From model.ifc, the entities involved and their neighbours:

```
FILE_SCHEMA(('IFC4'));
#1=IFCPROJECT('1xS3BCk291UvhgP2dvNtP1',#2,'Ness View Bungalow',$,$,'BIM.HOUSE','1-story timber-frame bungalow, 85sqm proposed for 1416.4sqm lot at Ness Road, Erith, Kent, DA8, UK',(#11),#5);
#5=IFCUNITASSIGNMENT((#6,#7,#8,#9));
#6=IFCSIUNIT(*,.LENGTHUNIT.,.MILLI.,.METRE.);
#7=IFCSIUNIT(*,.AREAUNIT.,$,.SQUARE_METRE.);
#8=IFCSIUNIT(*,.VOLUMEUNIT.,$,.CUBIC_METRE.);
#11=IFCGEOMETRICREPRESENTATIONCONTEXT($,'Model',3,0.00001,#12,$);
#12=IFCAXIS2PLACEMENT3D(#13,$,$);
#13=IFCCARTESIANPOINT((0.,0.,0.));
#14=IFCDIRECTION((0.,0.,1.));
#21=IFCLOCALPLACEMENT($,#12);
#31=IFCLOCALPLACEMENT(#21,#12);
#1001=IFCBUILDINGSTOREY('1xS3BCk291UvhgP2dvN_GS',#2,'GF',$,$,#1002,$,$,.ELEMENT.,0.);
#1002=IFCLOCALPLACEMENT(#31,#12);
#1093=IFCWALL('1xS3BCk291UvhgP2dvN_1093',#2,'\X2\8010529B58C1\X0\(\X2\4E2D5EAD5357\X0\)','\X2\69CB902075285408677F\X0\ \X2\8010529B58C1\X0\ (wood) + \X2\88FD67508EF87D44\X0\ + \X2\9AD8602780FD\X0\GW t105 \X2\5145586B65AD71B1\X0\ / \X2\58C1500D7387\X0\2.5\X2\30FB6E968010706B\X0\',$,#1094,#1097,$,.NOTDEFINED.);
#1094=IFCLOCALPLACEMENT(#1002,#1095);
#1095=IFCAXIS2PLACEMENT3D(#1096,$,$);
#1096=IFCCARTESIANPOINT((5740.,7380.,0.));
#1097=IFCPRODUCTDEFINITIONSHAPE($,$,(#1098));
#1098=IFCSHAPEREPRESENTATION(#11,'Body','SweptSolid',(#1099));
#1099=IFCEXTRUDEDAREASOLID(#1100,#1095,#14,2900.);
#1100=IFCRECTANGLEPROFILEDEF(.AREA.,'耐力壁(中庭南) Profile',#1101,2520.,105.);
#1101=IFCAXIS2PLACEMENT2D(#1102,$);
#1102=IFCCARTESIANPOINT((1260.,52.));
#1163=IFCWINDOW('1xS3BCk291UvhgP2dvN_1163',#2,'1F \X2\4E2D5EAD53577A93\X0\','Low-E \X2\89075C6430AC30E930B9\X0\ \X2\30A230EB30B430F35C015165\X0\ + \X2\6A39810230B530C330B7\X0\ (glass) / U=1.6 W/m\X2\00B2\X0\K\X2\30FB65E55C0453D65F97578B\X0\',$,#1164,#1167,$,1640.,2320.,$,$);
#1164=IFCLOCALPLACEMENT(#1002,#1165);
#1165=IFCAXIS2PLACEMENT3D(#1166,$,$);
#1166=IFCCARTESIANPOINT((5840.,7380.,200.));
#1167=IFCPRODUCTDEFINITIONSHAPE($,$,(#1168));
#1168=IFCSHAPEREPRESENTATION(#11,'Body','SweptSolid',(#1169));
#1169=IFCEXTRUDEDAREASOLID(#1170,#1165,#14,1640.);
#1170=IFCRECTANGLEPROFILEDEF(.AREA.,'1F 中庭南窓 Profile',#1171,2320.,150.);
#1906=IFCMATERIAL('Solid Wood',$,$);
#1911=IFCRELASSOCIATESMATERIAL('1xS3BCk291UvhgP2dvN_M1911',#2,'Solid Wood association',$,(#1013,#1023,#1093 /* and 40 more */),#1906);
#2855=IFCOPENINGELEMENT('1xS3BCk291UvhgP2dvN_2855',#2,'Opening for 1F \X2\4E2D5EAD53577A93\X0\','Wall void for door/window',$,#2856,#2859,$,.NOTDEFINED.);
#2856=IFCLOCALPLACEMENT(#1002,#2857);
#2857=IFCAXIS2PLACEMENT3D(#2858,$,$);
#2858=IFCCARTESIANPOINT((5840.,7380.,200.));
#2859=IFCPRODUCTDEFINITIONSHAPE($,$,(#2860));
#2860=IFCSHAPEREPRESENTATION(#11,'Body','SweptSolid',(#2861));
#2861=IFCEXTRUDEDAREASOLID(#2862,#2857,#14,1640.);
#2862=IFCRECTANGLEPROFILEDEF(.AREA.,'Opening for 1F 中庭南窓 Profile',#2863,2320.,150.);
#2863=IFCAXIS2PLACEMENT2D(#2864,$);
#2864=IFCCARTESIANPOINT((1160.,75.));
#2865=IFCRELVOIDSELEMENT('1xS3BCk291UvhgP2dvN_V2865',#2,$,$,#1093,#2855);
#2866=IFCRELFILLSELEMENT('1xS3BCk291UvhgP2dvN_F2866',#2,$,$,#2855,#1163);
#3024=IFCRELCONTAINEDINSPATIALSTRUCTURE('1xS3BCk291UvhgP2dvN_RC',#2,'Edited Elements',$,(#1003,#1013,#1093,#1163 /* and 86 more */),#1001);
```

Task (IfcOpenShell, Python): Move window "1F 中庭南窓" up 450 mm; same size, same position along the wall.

```python
import numpy as np
import ifcopenshell
import ifcopenshell.api.geometry
import ifcopenshell.util.placement
import ifcopenshell.util.unit

model = ifcopenshell.open("model.ifc")
unit_scale = ifcopenshell.util.unit.calculate_unit_scale(model)

window = model.by_guid("1xS3BCk291UvhgP2dvN_1163")
opening = window.FillsVoids[0].RelatingOpeningElement
dz = 0.45 / unit_scale

shift = np.array([0.0, 0.0, dz])
# The window is not placed relative to its opening, so move both.
for product in (opening, window):
    matrix = ifcopenshell.util.placement.get_local_placement(product.ObjectPlacement)
    matrix[:3, 3] += shift
    ifcopenshell.api.geometry.edit_object_placement(model, product=product, matrix=matrix, is_si=False)

print(f"moved by {dz * unit_scale:+.3f} m")

model.write("model_edited.ifc")
```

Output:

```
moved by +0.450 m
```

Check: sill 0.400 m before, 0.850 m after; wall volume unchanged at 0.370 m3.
